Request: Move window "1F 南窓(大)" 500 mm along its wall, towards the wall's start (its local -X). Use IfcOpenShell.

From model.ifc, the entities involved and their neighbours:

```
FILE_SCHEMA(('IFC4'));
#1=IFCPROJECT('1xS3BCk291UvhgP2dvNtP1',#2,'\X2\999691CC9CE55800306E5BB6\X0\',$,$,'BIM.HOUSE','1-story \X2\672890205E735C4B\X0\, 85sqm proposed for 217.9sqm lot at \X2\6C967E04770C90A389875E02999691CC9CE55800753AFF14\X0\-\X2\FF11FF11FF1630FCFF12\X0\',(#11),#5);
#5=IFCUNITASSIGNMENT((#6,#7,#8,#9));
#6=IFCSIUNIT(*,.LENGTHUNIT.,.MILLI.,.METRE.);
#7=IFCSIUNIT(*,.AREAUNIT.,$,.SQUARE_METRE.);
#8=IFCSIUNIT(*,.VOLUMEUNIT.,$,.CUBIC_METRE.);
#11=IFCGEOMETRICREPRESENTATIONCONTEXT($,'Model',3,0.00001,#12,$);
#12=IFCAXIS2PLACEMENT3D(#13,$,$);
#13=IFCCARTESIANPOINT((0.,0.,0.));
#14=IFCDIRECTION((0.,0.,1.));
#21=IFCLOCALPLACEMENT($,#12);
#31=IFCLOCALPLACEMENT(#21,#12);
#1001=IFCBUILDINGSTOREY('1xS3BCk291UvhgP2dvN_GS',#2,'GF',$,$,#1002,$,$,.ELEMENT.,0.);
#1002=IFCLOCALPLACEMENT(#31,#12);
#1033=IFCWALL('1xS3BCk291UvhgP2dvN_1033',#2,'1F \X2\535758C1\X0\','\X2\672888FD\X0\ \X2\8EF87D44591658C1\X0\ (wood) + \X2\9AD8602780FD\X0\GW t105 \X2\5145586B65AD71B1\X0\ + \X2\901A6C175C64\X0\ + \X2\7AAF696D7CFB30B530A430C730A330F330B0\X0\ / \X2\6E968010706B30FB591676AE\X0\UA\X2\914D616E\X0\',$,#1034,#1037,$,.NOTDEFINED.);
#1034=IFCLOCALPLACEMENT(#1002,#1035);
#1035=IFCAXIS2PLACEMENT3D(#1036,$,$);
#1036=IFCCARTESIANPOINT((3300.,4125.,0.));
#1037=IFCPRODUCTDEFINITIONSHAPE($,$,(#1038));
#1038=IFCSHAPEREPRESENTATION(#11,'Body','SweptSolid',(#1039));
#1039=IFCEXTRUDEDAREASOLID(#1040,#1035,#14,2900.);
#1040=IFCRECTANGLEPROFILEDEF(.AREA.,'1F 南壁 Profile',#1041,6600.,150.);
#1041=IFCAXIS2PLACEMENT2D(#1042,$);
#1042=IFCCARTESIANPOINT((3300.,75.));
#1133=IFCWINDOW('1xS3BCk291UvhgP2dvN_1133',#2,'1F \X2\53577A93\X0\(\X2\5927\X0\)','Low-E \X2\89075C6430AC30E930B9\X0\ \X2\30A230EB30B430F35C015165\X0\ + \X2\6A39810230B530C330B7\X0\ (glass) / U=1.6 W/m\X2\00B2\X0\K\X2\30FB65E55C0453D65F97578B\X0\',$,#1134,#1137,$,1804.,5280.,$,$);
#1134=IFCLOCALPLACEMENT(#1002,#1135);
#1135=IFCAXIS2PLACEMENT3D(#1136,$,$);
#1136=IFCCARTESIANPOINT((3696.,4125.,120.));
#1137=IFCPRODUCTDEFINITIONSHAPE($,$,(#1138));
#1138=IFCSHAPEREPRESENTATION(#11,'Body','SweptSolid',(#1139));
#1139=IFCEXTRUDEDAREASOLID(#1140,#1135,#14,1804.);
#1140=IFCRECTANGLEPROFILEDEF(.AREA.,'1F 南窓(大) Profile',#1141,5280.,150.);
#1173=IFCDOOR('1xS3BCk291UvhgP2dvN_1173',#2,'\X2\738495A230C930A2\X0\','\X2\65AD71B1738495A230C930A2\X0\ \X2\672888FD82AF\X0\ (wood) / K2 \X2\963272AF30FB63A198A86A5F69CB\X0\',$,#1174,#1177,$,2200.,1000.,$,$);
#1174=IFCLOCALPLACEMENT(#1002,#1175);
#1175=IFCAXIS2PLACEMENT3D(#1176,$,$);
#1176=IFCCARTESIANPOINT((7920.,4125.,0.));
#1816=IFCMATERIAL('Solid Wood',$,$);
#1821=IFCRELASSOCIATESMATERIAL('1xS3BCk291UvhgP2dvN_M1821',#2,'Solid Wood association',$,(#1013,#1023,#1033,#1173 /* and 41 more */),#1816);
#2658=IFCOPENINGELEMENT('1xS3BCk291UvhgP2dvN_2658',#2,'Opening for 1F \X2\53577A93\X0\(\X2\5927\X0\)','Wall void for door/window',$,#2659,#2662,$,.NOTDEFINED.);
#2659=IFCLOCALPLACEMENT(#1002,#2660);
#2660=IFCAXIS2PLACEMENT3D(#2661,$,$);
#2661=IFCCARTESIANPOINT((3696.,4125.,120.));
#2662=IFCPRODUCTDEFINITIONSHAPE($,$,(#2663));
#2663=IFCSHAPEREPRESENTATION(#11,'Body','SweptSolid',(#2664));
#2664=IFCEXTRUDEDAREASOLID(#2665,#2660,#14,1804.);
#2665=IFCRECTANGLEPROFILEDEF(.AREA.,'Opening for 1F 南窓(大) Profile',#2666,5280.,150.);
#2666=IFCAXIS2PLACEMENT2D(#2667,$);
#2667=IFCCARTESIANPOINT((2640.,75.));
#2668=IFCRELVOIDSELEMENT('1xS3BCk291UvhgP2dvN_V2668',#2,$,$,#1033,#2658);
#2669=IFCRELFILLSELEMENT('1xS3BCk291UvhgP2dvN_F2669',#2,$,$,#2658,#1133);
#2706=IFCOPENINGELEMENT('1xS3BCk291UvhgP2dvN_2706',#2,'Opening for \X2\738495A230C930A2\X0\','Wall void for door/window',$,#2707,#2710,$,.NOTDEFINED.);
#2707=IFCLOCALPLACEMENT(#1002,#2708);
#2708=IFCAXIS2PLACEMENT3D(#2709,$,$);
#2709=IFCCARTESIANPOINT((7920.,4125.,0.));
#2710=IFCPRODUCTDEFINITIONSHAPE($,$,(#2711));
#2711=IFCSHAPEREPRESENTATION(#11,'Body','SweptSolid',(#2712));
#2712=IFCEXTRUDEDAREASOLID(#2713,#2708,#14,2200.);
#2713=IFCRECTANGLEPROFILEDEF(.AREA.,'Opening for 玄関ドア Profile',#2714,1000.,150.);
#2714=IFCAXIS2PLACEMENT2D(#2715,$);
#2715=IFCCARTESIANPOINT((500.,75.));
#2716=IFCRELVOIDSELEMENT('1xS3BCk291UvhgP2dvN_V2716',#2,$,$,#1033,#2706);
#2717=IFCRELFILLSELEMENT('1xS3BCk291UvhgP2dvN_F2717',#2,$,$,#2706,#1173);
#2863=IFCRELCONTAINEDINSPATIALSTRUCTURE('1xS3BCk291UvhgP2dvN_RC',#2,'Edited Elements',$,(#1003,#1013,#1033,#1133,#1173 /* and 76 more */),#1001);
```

```python
import ifcopenshell
import ifcopenshell.api.geometry
import ifcopenshell.util.placement
import ifcopenshell.util.unit

model = ifcopenshell.open("model.ifc")
unit_scale = ifcopenshell.util.unit.calculate_unit_scale(model)

window = model.by_guid("1xS3BCk291UvhgP2dvN_1133")
opening = window.FillsVoids[0].RelatingOpeningElement
wall = opening.VoidsElements[0].RelatingBuildingElement

wall_matrix = ifcopenshell.util.placement.get_local_placement(wall.ObjectPlacement)
shift = wall_matrix[:3, 0] * -0.5 / unit_scale
before = ifcopenshell.util.placement.get_local_placement(window.ObjectPlacement)[:3, 3].copy()

# The window is not placed relative to its opening, so move both.
for product in (opening, window):
    matrix = ifcopenshell.util.placement.get_local_placement(product.ObjectPlacement)
    matrix[:3, 3] += shift
    ifcopenshell.api.geometry.edit_object_placement(model, product=product, matrix=matrix, is_si=False)

after = ifcopenshell.util.placement.get_local_placement(window.ObjectPlacement)[:3, 3]
print("window moved by", (after - before).round(3) + 0.0)

model.write("model_v2.ifc")
```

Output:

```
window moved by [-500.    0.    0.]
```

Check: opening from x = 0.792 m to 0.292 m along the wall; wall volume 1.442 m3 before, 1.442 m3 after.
